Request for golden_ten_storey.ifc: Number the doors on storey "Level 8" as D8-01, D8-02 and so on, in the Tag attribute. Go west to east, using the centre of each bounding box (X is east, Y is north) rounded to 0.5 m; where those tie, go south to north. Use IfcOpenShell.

First a look at what the model holds.

```python
import ifcopenshell
import ifcopenshell.util.element
import ifcopenshell.util.placement

model = ifcopenshell.open("golden_ten_storey.ifc")
print(model.schema)
storey = next(s for s in model.by_type("IfcBuildingStorey") if s.Name == "Level 8")
doors = [e for e in ifcopenshell.util.element.get_decomposition(storey) if e.is_a("IfcDoor")]
for e in sorted(doors, key=lambda e: e.id()):
    origin = ifcopenshell.util.placement.get_local_placement(e.ObjectPlacement)[:3, 3]
    print(e.id(), e.Tag, e.Name, origin.round(2) + 0.0, sep=" | ")
```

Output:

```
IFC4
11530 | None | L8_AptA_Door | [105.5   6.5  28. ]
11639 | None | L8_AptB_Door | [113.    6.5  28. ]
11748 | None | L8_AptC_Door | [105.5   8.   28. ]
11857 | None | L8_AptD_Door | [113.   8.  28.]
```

```python
import ifcopenshell
import ifcopenshell.geom
import ifcopenshell.util.element
import ifcopenshell.util.shape

model = ifcopenshell.open("golden_ten_storey.ifc")
settings = ifcopenshell.geom.settings()
settings.set("use-world-coords", True)


def centre(element):
    shape = ifcopenshell.geom.create_shape(settings, element)
    return ifcopenshell.util.shape.get_bbox_centroid(shape.geometry)


storey = next(s for s in model.by_type("IfcBuildingStorey") if s.Name == "Level 8")
doors = [e for e in ifcopenshell.util.element.get_decomposition(storey) if e.is_a("IfcDoor")]

# Insertion points can sit at a corner or the storey origin, so sort by the geometry (in metres).
centres = {e: centre(e) for e in doors}
doors.sort(key=lambda e: (round(centres[e][0] / 0.5), centres[e][1]))

for i, e in enumerate(doors, start=1):
    number = f"D8-{i:02d}"
    e.Tag = number
    print(e.id(), number)

model.write("golden_ten_storey_rev.ifc")
```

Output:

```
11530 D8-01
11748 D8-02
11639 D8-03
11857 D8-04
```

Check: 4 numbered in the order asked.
